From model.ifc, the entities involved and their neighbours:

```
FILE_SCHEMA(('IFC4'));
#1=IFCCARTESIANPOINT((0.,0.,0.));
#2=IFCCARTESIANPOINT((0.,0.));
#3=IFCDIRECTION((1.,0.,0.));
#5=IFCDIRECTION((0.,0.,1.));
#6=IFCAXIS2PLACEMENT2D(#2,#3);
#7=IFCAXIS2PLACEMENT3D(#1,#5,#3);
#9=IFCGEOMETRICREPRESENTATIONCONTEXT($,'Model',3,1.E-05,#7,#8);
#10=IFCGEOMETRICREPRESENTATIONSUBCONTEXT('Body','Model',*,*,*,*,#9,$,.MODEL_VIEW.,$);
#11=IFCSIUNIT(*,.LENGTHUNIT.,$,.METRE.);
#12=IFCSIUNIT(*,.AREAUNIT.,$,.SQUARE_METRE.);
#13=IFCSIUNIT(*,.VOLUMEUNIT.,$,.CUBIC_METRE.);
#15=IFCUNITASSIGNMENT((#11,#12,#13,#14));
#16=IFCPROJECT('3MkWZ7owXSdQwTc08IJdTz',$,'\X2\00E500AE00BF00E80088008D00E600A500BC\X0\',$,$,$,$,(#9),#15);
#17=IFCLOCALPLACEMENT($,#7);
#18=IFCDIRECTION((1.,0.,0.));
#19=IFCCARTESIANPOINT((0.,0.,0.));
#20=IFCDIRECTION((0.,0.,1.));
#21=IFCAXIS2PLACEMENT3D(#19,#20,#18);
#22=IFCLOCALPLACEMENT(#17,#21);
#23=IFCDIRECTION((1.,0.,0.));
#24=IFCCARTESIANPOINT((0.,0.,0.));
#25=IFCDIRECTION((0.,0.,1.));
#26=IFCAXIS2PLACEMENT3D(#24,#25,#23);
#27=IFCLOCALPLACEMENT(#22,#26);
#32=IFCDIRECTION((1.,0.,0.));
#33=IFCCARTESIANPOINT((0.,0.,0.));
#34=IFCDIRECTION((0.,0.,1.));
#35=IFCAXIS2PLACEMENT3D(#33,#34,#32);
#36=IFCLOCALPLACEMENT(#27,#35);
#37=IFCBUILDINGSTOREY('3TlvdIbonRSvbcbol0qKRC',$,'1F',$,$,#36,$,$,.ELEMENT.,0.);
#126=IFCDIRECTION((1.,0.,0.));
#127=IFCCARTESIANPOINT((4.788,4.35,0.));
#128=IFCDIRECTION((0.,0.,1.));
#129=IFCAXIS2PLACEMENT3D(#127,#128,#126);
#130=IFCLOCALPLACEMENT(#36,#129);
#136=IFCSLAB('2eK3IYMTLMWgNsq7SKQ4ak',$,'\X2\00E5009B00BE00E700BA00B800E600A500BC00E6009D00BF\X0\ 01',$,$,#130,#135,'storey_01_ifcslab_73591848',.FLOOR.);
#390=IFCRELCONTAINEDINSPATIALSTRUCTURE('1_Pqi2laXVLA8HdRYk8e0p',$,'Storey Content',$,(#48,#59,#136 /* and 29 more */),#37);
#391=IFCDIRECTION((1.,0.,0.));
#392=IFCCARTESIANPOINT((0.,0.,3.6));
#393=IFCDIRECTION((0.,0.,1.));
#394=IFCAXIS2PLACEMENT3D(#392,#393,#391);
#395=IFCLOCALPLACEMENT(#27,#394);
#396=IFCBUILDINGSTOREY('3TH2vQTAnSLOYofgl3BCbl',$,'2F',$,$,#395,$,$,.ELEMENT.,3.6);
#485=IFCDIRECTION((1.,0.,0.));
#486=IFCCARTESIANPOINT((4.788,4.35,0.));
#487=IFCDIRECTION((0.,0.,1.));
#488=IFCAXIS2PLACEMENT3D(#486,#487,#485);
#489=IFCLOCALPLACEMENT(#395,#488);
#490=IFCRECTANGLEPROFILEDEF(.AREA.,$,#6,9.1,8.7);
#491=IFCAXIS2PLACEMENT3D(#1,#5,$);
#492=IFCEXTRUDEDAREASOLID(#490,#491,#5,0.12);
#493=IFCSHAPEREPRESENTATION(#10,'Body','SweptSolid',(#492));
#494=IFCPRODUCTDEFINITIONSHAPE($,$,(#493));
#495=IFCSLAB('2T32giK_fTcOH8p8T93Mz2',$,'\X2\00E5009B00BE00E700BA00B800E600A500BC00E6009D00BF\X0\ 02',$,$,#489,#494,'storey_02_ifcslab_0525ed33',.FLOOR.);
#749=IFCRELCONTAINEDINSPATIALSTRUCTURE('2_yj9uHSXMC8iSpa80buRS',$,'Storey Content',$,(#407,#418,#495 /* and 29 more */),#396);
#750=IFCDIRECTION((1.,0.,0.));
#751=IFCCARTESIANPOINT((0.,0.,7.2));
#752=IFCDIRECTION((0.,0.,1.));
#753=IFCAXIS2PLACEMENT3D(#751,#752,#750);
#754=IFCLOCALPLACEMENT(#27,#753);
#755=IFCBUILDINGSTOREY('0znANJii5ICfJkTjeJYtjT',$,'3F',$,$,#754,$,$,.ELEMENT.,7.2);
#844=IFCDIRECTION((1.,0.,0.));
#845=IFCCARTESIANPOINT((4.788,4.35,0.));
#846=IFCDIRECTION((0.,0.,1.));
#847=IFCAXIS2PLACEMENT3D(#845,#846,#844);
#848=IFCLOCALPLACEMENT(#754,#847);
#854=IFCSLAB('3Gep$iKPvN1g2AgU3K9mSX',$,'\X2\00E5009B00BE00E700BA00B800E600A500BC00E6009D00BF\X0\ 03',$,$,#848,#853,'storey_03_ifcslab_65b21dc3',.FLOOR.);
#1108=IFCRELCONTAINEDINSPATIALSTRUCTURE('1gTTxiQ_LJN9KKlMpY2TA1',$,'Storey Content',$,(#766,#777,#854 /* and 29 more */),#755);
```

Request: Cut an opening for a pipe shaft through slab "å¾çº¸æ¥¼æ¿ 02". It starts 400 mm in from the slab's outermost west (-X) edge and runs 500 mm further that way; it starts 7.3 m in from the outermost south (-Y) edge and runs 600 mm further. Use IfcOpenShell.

```python
import numpy as np
import ifcopenshell
import ifcopenshell.api.feature
import ifcopenshell.api.geometry
import ifcopenshell.api.root
import ifcopenshell.geom
import ifcopenshell.util.placement
import ifcopenshell.util.representation
import ifcopenshell.util.shape
import ifcopenshell.util.unit

model = ifcopenshell.open("model.ifc")
unit_scale = ifcopenshell.util.unit.calculate_unit_scale(model)
settings = ifcopenshell.geom.settings()


def volume(element):
    """Net volume in cubic metres, openings subtracted."""
    shape = ifcopenshell.geom.create_shape(settings, element)
    return ifcopenshell.util.shape.get_volume(shape.geometry)


slab = model.by_guid("2T32giK_fTcOH8p8T93Mz2")
before = volume(slab)

# Extent in the slab's own axes, in metres. The edges named are its -X and -Y sides.
slab_shape = ifcopenshell.geom.create_shape(settings, slab)
vertices = ifcopenshell.util.shape.get_vertices(slab_shape.geometry)
x_min, y_min, bottom = vertices.min(axis=0)
top = vertices[:, 2].max()

opening = ifcopenshell.api.root.create_entity(model, ifc_class="IfcOpeningElement", name="Pipe shaft opening", predefined_type="OPENING")
context = ifcopenshell.util.representation.get_context(model, "Model", "Body", "MODEL_VIEW")
width, depth = 0.5, 0.6
outline = [(0.0, 0.0), (width, 0.0), (width, depth), (0.0, depth), (0.0, 0.0)]
# Overshoot both faces by 50 mm so the cut is clean.
shape = ifcopenshell.api.geometry.add_slab_representation(
    model, context=context, depth=top - bottom + 0.1, polyline=outline
)
ifcopenshell.api.geometry.assign_representation(model, product=opening, representation=shape)

matrix = ifcopenshell.util.placement.get_local_placement(slab.ObjectPlacement)
matrix[:, 3] = matrix @ np.append(np.array([x_min + 0.4, y_min + 7.3, bottom - 0.05]) / unit_scale, 1.0)
ifcopenshell.api.geometry.edit_object_placement(model, product=opening, matrix=matrix, is_si=False)
ifcopenshell.api.feature.add_feature(model, feature=opening, element=slab)

after = volume(slab)

print(f"slab volume {before:.3f} -> {after:.3f} m3")

model.write("model_edited.ifc")
```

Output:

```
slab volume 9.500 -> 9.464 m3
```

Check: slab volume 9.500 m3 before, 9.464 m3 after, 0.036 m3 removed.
